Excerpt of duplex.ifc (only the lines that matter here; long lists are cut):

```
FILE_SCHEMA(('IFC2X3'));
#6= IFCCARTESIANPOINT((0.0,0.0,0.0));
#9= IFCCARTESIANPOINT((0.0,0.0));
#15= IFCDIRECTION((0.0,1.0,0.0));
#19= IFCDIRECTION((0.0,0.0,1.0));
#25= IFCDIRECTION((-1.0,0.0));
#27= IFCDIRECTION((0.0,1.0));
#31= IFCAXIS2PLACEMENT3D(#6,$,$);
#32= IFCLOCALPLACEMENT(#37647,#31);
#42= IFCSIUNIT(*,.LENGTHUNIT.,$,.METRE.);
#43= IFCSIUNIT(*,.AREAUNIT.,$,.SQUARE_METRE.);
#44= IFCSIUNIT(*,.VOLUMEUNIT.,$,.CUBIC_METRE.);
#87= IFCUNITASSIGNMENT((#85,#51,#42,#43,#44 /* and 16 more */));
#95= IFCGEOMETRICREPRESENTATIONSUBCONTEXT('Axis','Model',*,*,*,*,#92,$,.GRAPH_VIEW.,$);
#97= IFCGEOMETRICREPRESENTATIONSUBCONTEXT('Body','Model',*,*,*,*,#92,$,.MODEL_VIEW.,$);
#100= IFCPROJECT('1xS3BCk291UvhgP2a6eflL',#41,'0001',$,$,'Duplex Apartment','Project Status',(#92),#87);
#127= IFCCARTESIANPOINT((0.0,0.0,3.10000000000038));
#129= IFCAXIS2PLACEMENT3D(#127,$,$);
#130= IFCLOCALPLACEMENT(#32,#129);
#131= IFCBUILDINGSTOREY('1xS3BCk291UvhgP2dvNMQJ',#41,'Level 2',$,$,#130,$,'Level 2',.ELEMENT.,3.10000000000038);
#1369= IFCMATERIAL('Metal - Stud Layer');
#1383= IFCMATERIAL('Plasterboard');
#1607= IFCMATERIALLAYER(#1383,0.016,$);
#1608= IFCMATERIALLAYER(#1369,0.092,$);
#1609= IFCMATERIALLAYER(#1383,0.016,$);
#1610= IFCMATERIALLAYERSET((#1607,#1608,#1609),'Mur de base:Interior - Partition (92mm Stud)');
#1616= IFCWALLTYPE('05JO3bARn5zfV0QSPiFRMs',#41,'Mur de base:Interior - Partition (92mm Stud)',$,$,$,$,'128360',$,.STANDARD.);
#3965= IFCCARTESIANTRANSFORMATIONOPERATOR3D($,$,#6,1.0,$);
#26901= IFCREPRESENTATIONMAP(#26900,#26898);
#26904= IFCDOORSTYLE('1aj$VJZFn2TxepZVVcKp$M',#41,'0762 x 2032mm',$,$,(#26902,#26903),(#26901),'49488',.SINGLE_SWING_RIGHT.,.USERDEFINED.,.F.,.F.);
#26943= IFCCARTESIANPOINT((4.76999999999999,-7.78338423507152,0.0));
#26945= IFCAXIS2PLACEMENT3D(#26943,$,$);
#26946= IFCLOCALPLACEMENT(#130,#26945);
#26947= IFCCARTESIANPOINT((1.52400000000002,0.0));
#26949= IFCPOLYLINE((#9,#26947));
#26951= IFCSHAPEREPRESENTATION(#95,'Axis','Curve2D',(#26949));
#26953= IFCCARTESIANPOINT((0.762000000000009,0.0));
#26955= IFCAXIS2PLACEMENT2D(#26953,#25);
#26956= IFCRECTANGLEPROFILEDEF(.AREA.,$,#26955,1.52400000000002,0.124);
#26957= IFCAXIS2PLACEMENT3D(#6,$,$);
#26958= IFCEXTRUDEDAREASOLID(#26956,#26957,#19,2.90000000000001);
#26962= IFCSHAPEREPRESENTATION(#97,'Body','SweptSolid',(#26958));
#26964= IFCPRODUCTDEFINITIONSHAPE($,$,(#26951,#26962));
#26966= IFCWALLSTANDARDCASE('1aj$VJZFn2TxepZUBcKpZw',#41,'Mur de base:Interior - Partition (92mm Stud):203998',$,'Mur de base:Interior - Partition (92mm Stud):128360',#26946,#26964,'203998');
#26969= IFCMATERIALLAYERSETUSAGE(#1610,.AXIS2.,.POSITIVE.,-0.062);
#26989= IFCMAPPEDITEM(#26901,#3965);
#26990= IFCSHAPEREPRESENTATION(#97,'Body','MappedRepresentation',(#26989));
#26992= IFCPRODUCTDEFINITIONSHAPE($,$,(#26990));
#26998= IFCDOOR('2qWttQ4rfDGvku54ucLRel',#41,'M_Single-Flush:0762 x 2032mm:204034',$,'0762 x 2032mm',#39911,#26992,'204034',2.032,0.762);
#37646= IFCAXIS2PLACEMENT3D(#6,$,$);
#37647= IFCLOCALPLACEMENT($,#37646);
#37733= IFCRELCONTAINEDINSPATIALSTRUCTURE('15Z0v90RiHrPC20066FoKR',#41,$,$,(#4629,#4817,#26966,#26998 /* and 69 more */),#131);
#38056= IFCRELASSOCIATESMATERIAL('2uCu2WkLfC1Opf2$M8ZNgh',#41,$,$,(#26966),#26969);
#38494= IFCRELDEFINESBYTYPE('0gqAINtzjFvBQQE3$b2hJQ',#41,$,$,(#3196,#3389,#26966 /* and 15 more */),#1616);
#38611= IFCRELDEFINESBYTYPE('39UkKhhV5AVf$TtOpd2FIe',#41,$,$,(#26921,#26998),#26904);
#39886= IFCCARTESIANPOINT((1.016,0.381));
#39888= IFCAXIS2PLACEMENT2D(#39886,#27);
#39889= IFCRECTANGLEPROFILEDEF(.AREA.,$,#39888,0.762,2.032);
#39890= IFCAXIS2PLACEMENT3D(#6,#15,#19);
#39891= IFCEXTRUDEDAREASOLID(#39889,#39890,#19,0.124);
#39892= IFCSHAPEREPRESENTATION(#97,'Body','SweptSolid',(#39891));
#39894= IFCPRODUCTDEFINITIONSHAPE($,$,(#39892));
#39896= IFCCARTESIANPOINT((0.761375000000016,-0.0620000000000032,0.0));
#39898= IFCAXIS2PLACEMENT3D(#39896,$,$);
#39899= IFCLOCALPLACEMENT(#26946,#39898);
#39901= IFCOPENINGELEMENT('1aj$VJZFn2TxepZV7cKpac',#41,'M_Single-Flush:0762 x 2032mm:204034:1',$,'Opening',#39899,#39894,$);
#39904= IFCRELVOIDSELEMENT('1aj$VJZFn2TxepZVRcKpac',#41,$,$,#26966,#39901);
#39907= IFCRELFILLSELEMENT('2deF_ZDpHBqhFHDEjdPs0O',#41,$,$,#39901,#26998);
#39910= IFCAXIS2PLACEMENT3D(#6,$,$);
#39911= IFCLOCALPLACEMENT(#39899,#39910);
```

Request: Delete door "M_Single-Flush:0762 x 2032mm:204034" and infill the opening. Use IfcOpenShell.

```python
import ifcopenshell
import ifcopenshell.api.feature
import ifcopenshell.api.root
import ifcopenshell.geom
import ifcopenshell.util.shape

model = ifcopenshell.open("duplex.ifc")
settings = ifcopenshell.geom.settings()


def volume(element):
    """Net volume in cubic metres, openings subtracted."""
    shape = ifcopenshell.geom.create_shape(settings, element)
    return ifcopenshell.util.shape.get_volume(shape.geometry)


door = model.by_guid("2qWttQ4rfDGvku54ucLRel")
opening = door.FillsVoids[0].RelatingOpeningElement
wall = opening.VoidsElements[0].RelatingBuildingElement
before = volume(wall)

ifcopenshell.api.root.remove_product(model, product=door)
ifcopenshell.api.feature.remove_feature(model, feature=opening)

after = volume(wall)

print(f"wall volume {before:.3f} -> {after:.3f} m3")

model.write("duplex-out.ifc")
```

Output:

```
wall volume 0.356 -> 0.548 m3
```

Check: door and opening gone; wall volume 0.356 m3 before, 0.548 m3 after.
